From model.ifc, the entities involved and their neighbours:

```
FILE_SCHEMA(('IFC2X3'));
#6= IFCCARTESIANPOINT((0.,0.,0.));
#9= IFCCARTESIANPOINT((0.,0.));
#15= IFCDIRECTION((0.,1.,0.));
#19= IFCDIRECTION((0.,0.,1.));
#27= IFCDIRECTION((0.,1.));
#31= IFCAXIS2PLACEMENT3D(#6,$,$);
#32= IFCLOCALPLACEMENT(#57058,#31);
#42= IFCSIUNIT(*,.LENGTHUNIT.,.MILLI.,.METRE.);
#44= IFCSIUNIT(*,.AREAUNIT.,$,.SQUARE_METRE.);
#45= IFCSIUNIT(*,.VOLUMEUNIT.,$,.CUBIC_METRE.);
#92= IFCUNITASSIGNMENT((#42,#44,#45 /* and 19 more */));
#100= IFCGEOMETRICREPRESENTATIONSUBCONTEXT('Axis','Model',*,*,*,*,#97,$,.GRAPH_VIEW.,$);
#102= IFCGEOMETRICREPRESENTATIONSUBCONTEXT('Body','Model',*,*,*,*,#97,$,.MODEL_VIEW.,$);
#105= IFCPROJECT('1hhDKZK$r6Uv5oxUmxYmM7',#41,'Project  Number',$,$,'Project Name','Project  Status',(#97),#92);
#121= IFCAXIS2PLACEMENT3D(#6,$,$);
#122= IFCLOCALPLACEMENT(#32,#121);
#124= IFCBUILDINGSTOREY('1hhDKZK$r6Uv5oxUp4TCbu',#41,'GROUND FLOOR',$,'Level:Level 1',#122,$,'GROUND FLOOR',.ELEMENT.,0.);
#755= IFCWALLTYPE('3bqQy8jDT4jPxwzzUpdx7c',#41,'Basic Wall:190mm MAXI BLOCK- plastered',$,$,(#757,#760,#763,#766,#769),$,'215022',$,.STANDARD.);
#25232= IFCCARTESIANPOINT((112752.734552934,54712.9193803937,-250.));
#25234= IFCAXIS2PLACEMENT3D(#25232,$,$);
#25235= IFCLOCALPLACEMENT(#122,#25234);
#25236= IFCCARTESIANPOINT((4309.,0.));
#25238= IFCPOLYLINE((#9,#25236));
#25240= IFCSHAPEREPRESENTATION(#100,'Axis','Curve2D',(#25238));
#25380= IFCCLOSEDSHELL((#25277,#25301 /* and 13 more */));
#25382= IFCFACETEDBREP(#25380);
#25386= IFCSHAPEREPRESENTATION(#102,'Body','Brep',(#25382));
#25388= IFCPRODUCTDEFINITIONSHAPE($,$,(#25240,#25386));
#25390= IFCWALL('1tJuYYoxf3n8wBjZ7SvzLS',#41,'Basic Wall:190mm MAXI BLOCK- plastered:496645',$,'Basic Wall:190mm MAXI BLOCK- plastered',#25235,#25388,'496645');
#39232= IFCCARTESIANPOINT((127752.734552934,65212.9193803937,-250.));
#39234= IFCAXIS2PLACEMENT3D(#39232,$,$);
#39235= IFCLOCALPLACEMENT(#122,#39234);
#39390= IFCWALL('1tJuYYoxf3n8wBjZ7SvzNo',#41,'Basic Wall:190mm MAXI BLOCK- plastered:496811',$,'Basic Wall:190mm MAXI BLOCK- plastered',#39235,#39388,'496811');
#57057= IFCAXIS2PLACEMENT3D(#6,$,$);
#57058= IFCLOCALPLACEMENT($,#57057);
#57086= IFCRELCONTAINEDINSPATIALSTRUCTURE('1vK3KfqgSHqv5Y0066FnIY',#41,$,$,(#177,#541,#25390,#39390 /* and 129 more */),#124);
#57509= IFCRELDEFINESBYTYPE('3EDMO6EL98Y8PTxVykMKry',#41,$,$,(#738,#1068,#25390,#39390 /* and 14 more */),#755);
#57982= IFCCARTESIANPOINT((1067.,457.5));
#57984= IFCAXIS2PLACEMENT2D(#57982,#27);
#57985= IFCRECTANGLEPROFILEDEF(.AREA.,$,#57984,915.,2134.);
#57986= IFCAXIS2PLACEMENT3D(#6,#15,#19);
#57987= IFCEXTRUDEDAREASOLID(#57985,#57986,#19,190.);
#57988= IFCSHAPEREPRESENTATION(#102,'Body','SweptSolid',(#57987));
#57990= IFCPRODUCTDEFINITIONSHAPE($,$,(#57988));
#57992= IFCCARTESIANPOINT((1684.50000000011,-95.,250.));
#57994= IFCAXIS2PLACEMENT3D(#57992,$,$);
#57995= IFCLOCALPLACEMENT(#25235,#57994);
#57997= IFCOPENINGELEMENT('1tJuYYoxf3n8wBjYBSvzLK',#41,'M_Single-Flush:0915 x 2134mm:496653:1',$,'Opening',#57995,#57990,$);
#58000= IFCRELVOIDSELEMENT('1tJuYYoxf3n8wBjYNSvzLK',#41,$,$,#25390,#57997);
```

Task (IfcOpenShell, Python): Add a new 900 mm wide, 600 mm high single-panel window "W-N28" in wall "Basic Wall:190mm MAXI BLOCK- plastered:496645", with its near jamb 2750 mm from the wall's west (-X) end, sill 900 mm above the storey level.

```python
import numpy as np
import ifcopenshell
import ifcopenshell.api.feature
import ifcopenshell.api.geometry
import ifcopenshell.api.root
import ifcopenshell.api.spatial
import ifcopenshell.api.type
import ifcopenshell.geom
import ifcopenshell.util.element
import ifcopenshell.util.placement
import ifcopenshell.util.representation
import ifcopenshell.util.shape
import ifcopenshell.util.unit

model = ifcopenshell.open("model.ifc")
unit_scale = ifcopenshell.util.unit.calculate_unit_scale(model)
settings = ifcopenshell.geom.settings()


def volume(element):
    """Net volume in cubic metres, openings subtracted."""
    shape = ifcopenshell.geom.create_shape(settings, element)
    return ifcopenshell.util.shape.get_volume(shape.geometry)


wall = model.by_guid("1tJuYYoxf3n8wBjZ7SvzLS")
storey = ifcopenshell.util.element.get_container(wall, ifc_class="IfcBuildingStorey")
context = ifcopenshell.util.representation.get_context(model, "Model", "Body", "MODEL_VIEW")
before = volume(wall)

width, height, from_end, sill = 0.9, 0.6, 2.75, 0.9  # metres

# The wall runs along its own X axis, and the end named is its -X end.
wall_shape = ifcopenshell.geom.create_shape(settings, wall)
x, y, z = ifcopenshell.util.shape.get_vertices(wall_shape.geometry).T
start = x.min() + from_end
face, thickness = float(y.min()), float(y.max() - y.min())
wall_matrix = ifcopenshell.util.placement.get_local_placement(wall.ObjectPlacement)
level = ifcopenshell.util.placement.get_local_placement(storey.ObjectPlacement)[2, 3]


def in_wall(x, y):
    """Placement at x, y metres in the wall's axes, at sill height."""
    matrix = wall_matrix.copy()
    matrix[:, 3] = wall_matrix @ np.array([x / unit_scale, y / unit_scale, 0.0, 1.0])
    matrix[2, 3] = level + sill / unit_scale
    return matrix


# Opening: a box that overshoots both wall faces by 50 mm.
opening = ifcopenshell.api.root.create_entity(model, ifc_class="IfcOpeningElement")
box = ifcopenshell.api.geometry.add_wall_representation(
    model, context=context, length=width, height=height, thickness=thickness + 0.1
)
ifcopenshell.api.geometry.assign_representation(model, product=opening, representation=box)
ifcopenshell.api.geometry.edit_object_placement(model, product=opening, matrix=in_wall(start, face - 0.05), is_si=False)
ifcopenshell.api.feature.add_feature(model, feature=opening, element=wall)

window = ifcopenshell.api.root.create_entity(model, ifc_class="IfcWindow", name="W-N28")
window.OverallWidth, window.OverallHeight = width / unit_scale, height / unit_scale
body = ifcopenshell.api.geometry.add_window_representation(
    model,
    context=context,
    overall_width=window.OverallWidth,
    overall_height=window.OverallHeight,
    partition_type="SINGLE_PANEL",
)
ifcopenshell.api.geometry.assign_representation(model, product=window, representation=body)
ifcopenshell.api.spatial.assign_container(model, products=[window], relating_structure=storey)
fills = ifcopenshell.api.feature.add_filling(model, opening=opening, element=window)
fills.OwnerHistory = window.OwnerHistory  # required in IFC2X3

# IFC2X3 keeps the operation on the window style.
style = ifcopenshell.api.root.create_entity(model, ifc_class="IfcWindowStyle", name="W-N28")
style.OperationType, style.ConstructionType = "SINGLE_PANEL", "NOTDEFINED"
style.ParameterTakesPrecedence = style.Sizeable = False
ifcopenshell.api.type.assign_type(model, related_objects=[window], relating_type=style)

# Centre the window in the wall's thickness.
ifcopenshell.api.geometry.edit_object_placement(model, product=window, matrix=in_wall(start, face), is_si=False)
window_shape = ifcopenshell.geom.create_shape(settings, window)
depth = ifcopenshell.util.shape.get_vertices(window_shape.geometry)[:, 1]
offset = face + thickness / 2 - (depth.min() + depth.max()) / 2
ifcopenshell.api.geometry.edit_object_placement(model, product=window, matrix=in_wall(start, offset), is_si=False)

after = volume(wall)

print(f"wall volume {before:.3f} -> {after:.3f} m3")

model.write("model_updated.ifc")
```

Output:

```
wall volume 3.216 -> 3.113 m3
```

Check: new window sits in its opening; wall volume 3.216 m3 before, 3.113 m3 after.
